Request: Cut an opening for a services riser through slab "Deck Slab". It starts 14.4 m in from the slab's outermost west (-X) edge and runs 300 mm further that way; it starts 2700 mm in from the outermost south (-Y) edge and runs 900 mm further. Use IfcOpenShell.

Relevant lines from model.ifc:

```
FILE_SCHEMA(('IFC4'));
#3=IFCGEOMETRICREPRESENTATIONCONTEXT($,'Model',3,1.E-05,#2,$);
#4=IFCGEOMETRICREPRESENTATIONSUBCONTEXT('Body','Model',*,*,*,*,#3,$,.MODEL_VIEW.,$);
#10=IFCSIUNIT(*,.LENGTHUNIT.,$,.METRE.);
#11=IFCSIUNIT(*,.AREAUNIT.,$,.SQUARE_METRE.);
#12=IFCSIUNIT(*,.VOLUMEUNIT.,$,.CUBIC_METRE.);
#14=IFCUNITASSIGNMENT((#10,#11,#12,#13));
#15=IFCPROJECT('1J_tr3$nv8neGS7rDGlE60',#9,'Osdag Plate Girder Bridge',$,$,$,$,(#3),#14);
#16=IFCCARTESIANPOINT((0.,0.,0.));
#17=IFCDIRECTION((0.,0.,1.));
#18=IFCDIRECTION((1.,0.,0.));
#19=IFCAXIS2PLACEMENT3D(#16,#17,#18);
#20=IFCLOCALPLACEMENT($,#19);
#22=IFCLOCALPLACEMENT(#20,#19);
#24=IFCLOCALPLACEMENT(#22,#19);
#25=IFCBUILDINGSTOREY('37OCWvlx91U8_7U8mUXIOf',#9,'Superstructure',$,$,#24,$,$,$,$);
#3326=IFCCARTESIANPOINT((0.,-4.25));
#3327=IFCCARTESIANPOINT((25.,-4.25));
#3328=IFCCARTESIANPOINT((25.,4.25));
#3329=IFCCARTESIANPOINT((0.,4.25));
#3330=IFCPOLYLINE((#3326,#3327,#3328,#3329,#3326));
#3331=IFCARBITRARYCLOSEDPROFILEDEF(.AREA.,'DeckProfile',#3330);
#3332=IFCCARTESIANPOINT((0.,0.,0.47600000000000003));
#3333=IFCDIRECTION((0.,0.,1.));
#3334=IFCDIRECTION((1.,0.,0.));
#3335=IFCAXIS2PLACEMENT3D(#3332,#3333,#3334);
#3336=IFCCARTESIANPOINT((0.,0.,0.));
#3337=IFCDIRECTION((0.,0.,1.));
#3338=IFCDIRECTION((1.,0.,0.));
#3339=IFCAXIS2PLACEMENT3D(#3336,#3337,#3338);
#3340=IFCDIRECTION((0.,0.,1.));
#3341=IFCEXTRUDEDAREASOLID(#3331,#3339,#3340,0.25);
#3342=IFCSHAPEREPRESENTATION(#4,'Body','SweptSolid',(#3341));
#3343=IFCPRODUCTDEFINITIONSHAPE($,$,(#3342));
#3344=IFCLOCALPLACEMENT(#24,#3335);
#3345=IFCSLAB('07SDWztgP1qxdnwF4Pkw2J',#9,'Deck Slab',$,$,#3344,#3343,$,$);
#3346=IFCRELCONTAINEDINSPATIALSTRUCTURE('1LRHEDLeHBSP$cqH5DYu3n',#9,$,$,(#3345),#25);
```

```python
import numpy as np
import ifcopenshell
import ifcopenshell.api.feature
import ifcopenshell.api.geometry
import ifcopenshell.api.root
import ifcopenshell.geom
import ifcopenshell.util.placement
import ifcopenshell.util.representation
import ifcopenshell.util.shape
import ifcopenshell.util.unit

model = ifcopenshell.open("model.ifc")
unit_scale = ifcopenshell.util.unit.calculate_unit_scale(model)
settings = ifcopenshell.geom.settings()


def volume(element):
    """Net volume in cubic metres, openings subtracted."""
    shape = ifcopenshell.geom.create_shape(settings, element)
    return ifcopenshell.util.shape.get_volume(shape.geometry)


slab = model.by_guid("07SDWztgP1qxdnwF4Pkw2J")
before = volume(slab)

# Extent in the slab's own axes, in metres. The edges named are its -X and -Y sides.
slab_shape = ifcopenshell.geom.create_shape(settings, slab)
vertices = ifcopenshell.util.shape.get_vertices(slab_shape.geometry)
x_min, y_min, bottom = vertices.min(axis=0)
top = vertices[:, 2].max()

opening = ifcopenshell.api.root.create_entity(model, ifc_class="IfcOpeningElement", name="Services riser opening", predefined_type="OPENING")
context = ifcopenshell.util.representation.get_context(model, "Model", "Body", "MODEL_VIEW")
width, depth = 0.3, 0.9
outline = [(0.0, 0.0), (width, 0.0), (width, depth), (0.0, depth), (0.0, 0.0)]
# Overshoot both faces by 50 mm so the cut is clean.
shape = ifcopenshell.api.geometry.add_slab_representation(
    model, context=context, depth=top - bottom + 0.1, polyline=outline
)
ifcopenshell.api.geometry.assign_representation(model, product=opening, representation=shape)

matrix = ifcopenshell.util.placement.get_local_placement(slab.ObjectPlacement)
matrix[:, 3] = matrix @ np.append(np.array([x_min + 14.4, y_min + 2.7, bottom - 0.05]) / unit_scale, 1.0)
ifcopenshell.api.geometry.edit_object_placement(model, product=opening, matrix=matrix, is_si=False)
ifcopenshell.api.feature.add_feature(model, feature=opening, element=slab)

after = volume(slab)

print(f"slab volume {before:.3f} -> {after:.3f} m3")

model.write("model-out.ifc")
```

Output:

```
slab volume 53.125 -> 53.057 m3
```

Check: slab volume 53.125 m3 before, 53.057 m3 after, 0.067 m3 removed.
